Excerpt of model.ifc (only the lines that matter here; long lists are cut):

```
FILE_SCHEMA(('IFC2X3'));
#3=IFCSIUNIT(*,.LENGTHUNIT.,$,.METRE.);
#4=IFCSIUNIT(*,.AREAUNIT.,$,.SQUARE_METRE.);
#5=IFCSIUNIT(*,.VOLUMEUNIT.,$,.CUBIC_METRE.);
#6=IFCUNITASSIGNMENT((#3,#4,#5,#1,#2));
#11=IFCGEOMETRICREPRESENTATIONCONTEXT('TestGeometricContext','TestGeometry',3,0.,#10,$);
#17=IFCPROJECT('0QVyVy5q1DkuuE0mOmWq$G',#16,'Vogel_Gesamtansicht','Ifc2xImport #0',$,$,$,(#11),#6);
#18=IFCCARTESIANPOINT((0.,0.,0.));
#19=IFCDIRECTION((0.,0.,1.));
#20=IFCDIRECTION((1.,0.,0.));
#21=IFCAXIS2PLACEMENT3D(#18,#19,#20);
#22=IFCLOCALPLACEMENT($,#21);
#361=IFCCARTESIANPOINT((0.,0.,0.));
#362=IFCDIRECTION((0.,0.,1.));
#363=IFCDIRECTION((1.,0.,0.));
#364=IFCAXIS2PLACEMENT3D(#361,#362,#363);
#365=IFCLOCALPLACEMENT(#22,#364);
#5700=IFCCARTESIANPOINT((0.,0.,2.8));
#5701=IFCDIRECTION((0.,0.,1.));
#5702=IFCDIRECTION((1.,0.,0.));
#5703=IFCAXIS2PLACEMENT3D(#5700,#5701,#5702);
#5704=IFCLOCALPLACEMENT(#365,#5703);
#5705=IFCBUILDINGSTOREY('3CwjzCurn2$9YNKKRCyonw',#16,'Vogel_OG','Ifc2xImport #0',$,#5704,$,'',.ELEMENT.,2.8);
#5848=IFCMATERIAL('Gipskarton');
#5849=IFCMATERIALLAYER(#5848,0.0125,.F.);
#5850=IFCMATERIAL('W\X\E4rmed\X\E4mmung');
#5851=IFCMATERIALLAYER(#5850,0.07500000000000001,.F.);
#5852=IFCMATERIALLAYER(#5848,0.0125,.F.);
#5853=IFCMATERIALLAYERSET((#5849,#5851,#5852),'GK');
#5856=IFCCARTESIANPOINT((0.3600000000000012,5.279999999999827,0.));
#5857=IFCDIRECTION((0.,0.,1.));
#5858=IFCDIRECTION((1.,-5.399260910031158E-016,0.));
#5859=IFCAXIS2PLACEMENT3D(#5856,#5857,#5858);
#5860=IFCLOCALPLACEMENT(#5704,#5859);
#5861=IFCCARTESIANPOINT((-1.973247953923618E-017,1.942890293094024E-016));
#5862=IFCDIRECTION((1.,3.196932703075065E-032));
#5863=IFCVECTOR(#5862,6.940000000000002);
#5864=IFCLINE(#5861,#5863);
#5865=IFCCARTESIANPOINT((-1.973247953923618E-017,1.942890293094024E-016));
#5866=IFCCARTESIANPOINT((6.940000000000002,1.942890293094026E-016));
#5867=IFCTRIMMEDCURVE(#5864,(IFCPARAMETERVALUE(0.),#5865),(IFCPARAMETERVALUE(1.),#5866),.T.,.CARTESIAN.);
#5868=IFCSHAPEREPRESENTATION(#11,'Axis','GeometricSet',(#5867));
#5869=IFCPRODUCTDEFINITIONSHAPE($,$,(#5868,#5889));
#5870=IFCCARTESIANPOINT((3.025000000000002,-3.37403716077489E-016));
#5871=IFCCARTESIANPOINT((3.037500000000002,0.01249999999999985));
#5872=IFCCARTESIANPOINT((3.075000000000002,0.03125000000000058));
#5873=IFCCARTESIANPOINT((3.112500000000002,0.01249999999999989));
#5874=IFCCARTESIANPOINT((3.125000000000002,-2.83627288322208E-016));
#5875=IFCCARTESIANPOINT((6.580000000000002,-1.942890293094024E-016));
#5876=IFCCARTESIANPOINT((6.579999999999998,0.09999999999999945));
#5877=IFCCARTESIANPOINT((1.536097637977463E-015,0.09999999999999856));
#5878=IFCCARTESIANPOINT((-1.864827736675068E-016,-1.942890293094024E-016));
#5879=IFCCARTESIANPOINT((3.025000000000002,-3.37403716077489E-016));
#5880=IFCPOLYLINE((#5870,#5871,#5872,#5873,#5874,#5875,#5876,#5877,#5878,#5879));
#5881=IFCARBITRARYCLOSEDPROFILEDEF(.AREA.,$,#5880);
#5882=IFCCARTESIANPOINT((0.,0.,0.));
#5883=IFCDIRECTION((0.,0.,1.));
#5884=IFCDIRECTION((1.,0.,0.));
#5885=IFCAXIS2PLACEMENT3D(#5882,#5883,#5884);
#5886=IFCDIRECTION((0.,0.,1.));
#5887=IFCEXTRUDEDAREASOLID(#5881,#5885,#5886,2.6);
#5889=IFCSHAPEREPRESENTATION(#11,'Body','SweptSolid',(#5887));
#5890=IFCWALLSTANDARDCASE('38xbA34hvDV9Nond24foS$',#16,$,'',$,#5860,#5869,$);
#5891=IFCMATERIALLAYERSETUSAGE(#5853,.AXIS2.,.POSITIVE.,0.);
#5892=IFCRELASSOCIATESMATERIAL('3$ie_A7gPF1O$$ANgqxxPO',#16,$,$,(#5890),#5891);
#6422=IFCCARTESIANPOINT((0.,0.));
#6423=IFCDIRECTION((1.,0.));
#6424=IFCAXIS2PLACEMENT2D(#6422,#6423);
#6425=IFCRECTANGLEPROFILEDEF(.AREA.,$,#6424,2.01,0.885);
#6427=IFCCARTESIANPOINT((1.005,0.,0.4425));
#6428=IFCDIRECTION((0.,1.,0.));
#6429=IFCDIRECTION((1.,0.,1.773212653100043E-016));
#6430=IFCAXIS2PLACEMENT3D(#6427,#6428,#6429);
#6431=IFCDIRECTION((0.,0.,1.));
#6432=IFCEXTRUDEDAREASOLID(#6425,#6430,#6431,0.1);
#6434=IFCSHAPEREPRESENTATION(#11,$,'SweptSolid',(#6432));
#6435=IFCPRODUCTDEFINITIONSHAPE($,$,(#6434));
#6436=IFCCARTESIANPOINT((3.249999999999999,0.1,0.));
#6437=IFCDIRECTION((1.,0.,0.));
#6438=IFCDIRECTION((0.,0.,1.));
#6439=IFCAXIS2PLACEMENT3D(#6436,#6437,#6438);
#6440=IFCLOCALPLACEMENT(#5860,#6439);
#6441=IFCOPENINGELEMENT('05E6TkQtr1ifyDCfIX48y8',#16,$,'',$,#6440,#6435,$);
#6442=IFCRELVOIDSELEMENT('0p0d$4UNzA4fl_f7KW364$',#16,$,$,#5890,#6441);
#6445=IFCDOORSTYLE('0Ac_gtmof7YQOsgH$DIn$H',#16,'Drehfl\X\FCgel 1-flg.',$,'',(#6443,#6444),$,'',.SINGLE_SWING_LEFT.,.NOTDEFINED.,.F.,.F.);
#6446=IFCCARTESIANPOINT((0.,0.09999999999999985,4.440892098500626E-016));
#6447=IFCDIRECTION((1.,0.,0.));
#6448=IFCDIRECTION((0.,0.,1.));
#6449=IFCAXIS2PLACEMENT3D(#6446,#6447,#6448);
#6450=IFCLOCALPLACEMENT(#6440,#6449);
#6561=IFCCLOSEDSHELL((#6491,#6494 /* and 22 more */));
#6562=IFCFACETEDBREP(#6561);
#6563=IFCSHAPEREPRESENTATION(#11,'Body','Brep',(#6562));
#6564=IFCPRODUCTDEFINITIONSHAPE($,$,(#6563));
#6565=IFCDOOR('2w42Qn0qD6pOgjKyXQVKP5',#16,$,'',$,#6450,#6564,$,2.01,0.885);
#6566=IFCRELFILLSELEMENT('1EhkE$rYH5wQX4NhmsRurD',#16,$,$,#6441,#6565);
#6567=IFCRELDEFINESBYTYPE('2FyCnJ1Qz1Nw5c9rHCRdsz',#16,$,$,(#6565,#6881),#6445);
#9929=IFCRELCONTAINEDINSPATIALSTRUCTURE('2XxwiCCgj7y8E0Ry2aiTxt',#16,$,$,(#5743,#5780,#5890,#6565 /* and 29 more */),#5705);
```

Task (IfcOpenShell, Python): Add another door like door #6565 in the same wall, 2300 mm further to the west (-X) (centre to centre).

```python
import ifcopenshell
import ifcopenshell.api.feature
import ifcopenshell.api.geometry
import ifcopenshell.api.root
import ifcopenshell.geom
import ifcopenshell.util.element
import ifcopenshell.util.placement
import ifcopenshell.util.shape
import ifcopenshell.util.unit

model = ifcopenshell.open("model.ifc")
unit_scale = ifcopenshell.util.unit.calculate_unit_scale(model)
settings = ifcopenshell.geom.settings()


def volume(element):
    """Net volume in cubic metres, openings subtracted."""
    shape = ifcopenshell.geom.create_shape(settings, element)
    return ifcopenshell.util.shape.get_volume(shape.geometry)


door = model.by_guid("2w42Qn0qD6pOgjKyXQVKP5")
opening = door.FillsVoids[0].RelatingOpeningElement
wall = opening.VoidsElements[0].RelatingBuildingElement
before = volume(wall)
shift = ifcopenshell.util.placement.get_local_placement(wall.ObjectPlacement)[:3, 0] * -2.3 / unit_scale

# copy_class copies the void relationship, type, container and properties, but no geometry.
new_opening = ifcopenshell.api.root.copy_class(model, product=opening)
new_opening.Representation = ifcopenshell.util.element.copy_deep(
    model, opening.Representation, exclude=["IfcGeometricRepresentationContext", "IfcRepresentationMap"]
)
new_door = ifcopenshell.api.root.copy_class(model, product=door)
new_door.Representation = ifcopenshell.util.element.copy_deep(
    model, door.Representation, exclude=["IfcGeometricRepresentationContext", "IfcRepresentationMap"]
)
fills = ifcopenshell.api.feature.add_filling(model, opening=new_opening, element=new_door)
fills.OwnerHistory = new_door.OwnerHistory  # required in IFC2X3

for old, new in ((opening, new_opening), (door, new_door)):
    matrix = ifcopenshell.util.placement.get_local_placement(old.ObjectPlacement)
    matrix[:3, 3] += shift
    ifcopenshell.api.geometry.edit_object_placement(model, product=new, matrix=matrix, is_si=False)

after = volume(wall)

print(f"wall volume {before:.3f} -> {after:.3f} m3")

model.write("model_edited.ifc")
```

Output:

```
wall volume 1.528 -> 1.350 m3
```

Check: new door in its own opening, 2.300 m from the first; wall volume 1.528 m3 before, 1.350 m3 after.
